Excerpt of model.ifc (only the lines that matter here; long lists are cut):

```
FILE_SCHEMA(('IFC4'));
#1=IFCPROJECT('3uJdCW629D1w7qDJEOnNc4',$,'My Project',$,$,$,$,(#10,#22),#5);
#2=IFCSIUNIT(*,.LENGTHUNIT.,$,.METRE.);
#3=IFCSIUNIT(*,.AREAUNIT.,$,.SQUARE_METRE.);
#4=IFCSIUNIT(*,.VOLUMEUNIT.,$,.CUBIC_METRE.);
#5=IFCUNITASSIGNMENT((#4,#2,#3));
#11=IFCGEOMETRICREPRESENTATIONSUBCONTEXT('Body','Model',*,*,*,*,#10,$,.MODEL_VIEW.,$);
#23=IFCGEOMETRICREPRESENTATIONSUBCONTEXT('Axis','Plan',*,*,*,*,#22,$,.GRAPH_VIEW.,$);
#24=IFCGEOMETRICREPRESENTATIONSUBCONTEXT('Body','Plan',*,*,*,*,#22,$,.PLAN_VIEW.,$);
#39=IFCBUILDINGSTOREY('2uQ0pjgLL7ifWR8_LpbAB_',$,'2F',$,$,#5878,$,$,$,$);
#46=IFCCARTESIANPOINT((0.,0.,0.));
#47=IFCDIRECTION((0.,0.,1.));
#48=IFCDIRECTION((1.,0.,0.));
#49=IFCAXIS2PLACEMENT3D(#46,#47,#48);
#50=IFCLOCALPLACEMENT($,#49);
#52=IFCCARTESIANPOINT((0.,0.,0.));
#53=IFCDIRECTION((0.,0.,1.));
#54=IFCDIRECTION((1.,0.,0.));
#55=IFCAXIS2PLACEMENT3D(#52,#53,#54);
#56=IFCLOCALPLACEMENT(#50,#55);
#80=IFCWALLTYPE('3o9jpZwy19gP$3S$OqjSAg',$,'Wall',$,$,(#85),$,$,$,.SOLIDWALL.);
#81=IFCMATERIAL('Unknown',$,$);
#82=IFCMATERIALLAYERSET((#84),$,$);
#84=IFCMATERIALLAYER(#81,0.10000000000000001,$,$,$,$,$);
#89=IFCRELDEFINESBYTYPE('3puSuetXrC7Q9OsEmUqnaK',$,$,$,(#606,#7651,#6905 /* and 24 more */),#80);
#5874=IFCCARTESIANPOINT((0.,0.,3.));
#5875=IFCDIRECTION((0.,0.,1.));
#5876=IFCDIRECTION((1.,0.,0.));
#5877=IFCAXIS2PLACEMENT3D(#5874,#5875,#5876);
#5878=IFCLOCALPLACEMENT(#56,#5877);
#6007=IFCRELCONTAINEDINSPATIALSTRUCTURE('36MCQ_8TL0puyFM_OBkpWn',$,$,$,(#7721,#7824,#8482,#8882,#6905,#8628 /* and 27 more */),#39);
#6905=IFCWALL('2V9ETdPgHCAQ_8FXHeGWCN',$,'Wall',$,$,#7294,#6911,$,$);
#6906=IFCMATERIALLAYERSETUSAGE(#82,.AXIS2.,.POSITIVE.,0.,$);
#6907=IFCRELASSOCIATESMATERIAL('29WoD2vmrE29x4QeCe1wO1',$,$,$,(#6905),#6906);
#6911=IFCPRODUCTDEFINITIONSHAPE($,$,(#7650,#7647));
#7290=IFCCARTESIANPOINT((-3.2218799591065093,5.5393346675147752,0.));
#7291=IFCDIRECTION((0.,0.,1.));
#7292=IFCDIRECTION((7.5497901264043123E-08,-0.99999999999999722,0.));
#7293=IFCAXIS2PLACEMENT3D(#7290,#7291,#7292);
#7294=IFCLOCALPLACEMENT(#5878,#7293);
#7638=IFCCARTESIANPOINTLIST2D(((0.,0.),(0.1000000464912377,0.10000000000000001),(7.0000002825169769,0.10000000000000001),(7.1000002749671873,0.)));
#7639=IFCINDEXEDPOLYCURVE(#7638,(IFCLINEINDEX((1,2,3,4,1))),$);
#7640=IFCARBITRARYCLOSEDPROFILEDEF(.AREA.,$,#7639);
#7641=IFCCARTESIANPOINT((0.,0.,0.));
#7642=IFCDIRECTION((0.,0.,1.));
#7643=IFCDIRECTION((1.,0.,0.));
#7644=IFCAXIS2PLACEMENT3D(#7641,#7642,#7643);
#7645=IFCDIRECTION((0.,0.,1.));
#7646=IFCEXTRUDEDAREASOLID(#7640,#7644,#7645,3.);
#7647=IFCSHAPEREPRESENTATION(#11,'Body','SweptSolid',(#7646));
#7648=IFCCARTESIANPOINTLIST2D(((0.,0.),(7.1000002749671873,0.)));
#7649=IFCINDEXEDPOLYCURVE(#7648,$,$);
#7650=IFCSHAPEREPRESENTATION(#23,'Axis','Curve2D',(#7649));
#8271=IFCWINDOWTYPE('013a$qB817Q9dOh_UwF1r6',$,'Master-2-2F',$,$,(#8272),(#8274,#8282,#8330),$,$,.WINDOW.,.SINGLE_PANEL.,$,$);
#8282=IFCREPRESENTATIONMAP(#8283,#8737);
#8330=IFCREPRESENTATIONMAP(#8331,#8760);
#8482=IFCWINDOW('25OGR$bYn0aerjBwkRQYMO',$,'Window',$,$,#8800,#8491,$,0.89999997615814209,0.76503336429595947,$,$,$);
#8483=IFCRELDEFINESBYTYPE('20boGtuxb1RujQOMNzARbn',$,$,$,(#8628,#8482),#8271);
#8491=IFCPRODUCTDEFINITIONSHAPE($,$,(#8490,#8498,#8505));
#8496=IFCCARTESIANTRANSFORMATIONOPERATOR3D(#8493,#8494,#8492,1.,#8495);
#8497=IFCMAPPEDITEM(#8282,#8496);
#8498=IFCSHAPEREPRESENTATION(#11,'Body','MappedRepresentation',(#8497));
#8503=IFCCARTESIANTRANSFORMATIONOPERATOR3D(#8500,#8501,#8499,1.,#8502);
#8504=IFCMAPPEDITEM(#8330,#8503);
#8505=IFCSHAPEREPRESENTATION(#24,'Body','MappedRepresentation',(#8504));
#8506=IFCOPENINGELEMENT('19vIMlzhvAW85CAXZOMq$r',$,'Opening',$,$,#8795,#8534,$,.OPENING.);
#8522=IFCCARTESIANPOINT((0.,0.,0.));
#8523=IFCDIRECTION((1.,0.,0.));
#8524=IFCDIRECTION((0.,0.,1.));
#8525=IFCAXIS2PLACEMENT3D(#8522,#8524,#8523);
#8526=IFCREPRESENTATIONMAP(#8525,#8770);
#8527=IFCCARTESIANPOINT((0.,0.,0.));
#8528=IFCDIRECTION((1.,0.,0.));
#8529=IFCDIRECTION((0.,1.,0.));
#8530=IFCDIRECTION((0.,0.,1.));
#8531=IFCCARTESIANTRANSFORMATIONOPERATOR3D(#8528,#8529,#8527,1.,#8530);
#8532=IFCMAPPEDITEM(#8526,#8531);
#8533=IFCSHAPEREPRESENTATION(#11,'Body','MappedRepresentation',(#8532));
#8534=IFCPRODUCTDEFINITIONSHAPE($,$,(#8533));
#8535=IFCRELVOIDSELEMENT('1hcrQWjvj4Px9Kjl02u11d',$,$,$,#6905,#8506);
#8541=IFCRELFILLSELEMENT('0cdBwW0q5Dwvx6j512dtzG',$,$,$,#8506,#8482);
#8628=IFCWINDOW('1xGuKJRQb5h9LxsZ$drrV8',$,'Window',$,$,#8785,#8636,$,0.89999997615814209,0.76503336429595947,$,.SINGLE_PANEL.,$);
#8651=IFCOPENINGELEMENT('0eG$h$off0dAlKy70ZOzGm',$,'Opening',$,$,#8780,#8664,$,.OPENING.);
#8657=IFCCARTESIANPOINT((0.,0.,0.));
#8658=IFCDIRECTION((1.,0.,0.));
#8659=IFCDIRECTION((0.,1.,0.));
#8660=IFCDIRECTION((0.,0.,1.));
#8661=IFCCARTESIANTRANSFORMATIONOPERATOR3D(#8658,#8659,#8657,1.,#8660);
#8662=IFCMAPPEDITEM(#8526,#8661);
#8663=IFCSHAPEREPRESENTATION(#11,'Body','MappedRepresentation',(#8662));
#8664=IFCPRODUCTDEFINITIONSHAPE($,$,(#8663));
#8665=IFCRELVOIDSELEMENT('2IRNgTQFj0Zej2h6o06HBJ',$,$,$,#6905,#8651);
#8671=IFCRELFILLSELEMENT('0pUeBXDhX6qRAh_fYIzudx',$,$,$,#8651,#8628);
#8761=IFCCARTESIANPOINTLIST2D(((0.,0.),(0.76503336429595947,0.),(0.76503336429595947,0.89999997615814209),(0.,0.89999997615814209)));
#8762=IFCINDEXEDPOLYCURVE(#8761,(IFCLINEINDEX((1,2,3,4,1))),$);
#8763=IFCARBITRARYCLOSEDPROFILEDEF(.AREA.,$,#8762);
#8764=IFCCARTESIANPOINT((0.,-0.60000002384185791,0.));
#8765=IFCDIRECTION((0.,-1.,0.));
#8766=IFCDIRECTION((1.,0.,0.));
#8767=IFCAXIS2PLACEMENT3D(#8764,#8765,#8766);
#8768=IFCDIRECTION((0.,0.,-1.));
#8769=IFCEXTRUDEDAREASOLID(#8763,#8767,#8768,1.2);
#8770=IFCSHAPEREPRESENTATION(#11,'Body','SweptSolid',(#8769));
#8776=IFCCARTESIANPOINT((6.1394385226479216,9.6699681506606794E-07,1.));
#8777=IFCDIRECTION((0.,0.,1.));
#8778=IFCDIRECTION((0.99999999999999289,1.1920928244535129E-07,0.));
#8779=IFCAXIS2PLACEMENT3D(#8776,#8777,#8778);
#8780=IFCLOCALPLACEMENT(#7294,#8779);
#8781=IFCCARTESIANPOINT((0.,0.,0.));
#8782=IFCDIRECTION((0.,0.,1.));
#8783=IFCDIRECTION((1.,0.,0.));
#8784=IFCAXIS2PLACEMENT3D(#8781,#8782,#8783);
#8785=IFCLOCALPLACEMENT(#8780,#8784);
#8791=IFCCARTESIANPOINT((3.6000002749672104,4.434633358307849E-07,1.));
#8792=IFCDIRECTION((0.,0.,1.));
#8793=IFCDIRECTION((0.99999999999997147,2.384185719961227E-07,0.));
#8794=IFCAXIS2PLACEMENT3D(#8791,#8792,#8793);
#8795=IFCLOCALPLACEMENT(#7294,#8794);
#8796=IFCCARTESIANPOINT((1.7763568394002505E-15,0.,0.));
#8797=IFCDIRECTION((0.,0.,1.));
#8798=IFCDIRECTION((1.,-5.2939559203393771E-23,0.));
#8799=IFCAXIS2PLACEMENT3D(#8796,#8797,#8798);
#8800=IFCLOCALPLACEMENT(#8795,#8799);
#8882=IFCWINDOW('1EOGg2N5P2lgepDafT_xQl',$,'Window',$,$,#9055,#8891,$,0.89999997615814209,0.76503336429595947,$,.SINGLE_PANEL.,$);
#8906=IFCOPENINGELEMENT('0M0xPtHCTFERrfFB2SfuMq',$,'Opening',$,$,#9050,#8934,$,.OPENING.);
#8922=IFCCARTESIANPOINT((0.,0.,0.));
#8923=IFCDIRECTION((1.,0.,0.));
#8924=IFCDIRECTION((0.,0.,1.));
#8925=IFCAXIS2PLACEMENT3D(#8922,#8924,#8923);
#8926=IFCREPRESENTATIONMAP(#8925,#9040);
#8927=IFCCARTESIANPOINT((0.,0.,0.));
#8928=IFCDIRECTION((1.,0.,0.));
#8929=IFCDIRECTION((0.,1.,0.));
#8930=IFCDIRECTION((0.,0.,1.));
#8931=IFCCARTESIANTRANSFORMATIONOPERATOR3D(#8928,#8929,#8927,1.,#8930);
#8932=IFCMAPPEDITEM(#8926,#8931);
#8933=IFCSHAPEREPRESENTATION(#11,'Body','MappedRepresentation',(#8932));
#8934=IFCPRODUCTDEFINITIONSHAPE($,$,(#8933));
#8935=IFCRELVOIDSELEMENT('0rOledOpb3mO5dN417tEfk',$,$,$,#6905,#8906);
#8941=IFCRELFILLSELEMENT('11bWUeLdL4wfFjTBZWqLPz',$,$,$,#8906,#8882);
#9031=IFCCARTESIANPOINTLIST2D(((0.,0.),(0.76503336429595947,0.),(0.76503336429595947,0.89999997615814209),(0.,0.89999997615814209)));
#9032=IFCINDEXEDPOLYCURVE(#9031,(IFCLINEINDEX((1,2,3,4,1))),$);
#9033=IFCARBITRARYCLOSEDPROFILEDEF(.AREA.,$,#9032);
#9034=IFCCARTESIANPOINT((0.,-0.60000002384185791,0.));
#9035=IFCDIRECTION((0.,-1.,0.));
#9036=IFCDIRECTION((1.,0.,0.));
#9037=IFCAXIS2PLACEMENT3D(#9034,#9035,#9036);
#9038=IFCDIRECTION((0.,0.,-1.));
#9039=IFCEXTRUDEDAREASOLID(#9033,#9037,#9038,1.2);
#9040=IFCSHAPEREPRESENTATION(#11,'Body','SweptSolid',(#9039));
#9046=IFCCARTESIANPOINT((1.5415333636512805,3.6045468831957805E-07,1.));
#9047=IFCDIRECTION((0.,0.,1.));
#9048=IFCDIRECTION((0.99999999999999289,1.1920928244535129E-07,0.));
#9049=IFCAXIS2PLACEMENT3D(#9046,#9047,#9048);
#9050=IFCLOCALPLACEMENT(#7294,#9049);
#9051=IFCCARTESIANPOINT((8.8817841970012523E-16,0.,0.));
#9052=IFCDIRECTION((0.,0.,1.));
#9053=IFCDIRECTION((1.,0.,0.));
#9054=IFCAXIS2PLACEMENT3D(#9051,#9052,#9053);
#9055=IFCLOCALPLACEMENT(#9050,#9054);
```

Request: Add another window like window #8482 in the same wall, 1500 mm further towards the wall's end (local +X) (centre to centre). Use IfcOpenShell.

```python
import ifcopenshell
import ifcopenshell.api.feature
import ifcopenshell.api.geometry
import ifcopenshell.api.root
import ifcopenshell.geom
import ifcopenshell.util.element
import ifcopenshell.util.placement
import ifcopenshell.util.shape

model = ifcopenshell.open("model.ifc")
settings = ifcopenshell.geom.settings()


def volume(element):
    """Net volume in cubic metres, openings subtracted."""
    shape = ifcopenshell.geom.create_shape(settings, element)
    return ifcopenshell.util.shape.get_volume(shape.geometry)


window = model.by_guid("25OGR$bYn0aerjBwkRQYMO")
opening = window.FillsVoids[0].RelatingOpeningElement
wall = opening.VoidsElements[0].RelatingBuildingElement
before = volume(wall)
shift = ifcopenshell.util.placement.get_local_placement(wall.ObjectPlacement)[:3, 0] * 1.5

# copy_class copies the void relationship, type, container and properties, but no geometry.
new_opening = ifcopenshell.api.root.copy_class(model, product=opening)
new_opening.Representation = ifcopenshell.util.element.copy_deep(
    model, opening.Representation, exclude=["IfcGeometricRepresentationContext", "IfcRepresentationMap"]
)
new_window = ifcopenshell.api.root.copy_class(model, product=window)
new_window.Representation = ifcopenshell.util.element.copy_deep(
    model, window.Representation, exclude=["IfcGeometricRepresentationContext", "IfcRepresentationMap"]
)
ifcopenshell.api.feature.add_filling(model, opening=new_opening, element=new_window)

for old, new in ((opening, new_opening), (window, new_window)):
    matrix = ifcopenshell.util.placement.get_local_placement(old.ObjectPlacement)
    matrix[:3, 3] += shift
    ifcopenshell.api.geometry.edit_object_placement(model, product=new, matrix=matrix, is_si=False)

after = volume(wall)

print(f"wall volume {before:.3f} -> {after:.3f} m3")

model.write("model_edited.ifc")
```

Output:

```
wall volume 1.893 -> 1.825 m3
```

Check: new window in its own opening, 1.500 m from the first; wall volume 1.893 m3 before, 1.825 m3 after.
